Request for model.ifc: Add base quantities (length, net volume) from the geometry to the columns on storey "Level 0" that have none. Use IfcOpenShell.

First a look at what the model holds.

```python
import ifcopenshell
import ifcopenshell.util.element
import ifcopenshell.util.unit

model = ifcopenshell.open("model.ifc")
print(model.schema)
for unit_type in ("LENGTHUNIT", "AREAUNIT", "VOLUMEUNIT"):
    print(unit_type, ifcopenshell.util.unit.calculate_unit_scale(model, unit_type))
storey = next(s for s in model.by_type("IfcBuildingStorey") if s.Name == "Level 0")
columns = [e for e in ifcopenshell.util.element.get_decomposition(storey) if e.is_a("IfcColumn")]
for e in sorted(columns, key=lambda e: e.id()):
    print(e.id(), e.is_a(), e.Name, list(ifcopenshell.util.element.get_psets(e, qtos_only=True)), sep=" | ")
```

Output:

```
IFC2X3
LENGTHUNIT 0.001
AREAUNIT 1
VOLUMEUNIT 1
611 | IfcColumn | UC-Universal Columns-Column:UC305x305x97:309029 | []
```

```python
import ifcopenshell
import ifcopenshell.api.pset
import ifcopenshell.geom
import ifcopenshell.util.element
import ifcopenshell.util.shape
import ifcopenshell.util.unit

model = ifcopenshell.open("model.ifc")
unit_scale = ifcopenshell.util.unit.calculate_unit_scale(model)
volume_scale = ifcopenshell.util.unit.calculate_unit_scale(model, "VOLUMEUNIT")
settings = ifcopenshell.geom.settings()

storey = next(s for s in model.by_type("IfcBuildingStorey") if s.Name == "Level 0")
columns = [e for e in ifcopenshell.util.element.get_decomposition(storey) if e.is_a("IfcColumn")]

for e in sorted(columns, key=lambda e: e.id()):
    if ifcopenshell.util.element.get_psets(e, qtos_only=True, should_inherit=False):
        continue
    # Geometry comes back in metres, in the element's own axes.
    shape = ifcopenshell.geom.create_shape(settings, e)
    values = {
        "Length": ifcopenshell.util.shape.get_z(shape.geometry) / unit_scale,
        "NetVolume": ifcopenshell.util.shape.get_volume(shape.geometry) / volume_scale,
    }
    qto = ifcopenshell.api.pset.add_qto(model, product=e, name="BaseQuantities")
    ifcopenshell.api.pset.edit_qto(model, qto=qto, properties=values)
    print(e.id(), {k: round(v, 3) for k, v in values.items()})

model.write("model_rev.ifc")
```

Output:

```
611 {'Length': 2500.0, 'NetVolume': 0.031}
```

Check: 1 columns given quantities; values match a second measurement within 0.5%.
